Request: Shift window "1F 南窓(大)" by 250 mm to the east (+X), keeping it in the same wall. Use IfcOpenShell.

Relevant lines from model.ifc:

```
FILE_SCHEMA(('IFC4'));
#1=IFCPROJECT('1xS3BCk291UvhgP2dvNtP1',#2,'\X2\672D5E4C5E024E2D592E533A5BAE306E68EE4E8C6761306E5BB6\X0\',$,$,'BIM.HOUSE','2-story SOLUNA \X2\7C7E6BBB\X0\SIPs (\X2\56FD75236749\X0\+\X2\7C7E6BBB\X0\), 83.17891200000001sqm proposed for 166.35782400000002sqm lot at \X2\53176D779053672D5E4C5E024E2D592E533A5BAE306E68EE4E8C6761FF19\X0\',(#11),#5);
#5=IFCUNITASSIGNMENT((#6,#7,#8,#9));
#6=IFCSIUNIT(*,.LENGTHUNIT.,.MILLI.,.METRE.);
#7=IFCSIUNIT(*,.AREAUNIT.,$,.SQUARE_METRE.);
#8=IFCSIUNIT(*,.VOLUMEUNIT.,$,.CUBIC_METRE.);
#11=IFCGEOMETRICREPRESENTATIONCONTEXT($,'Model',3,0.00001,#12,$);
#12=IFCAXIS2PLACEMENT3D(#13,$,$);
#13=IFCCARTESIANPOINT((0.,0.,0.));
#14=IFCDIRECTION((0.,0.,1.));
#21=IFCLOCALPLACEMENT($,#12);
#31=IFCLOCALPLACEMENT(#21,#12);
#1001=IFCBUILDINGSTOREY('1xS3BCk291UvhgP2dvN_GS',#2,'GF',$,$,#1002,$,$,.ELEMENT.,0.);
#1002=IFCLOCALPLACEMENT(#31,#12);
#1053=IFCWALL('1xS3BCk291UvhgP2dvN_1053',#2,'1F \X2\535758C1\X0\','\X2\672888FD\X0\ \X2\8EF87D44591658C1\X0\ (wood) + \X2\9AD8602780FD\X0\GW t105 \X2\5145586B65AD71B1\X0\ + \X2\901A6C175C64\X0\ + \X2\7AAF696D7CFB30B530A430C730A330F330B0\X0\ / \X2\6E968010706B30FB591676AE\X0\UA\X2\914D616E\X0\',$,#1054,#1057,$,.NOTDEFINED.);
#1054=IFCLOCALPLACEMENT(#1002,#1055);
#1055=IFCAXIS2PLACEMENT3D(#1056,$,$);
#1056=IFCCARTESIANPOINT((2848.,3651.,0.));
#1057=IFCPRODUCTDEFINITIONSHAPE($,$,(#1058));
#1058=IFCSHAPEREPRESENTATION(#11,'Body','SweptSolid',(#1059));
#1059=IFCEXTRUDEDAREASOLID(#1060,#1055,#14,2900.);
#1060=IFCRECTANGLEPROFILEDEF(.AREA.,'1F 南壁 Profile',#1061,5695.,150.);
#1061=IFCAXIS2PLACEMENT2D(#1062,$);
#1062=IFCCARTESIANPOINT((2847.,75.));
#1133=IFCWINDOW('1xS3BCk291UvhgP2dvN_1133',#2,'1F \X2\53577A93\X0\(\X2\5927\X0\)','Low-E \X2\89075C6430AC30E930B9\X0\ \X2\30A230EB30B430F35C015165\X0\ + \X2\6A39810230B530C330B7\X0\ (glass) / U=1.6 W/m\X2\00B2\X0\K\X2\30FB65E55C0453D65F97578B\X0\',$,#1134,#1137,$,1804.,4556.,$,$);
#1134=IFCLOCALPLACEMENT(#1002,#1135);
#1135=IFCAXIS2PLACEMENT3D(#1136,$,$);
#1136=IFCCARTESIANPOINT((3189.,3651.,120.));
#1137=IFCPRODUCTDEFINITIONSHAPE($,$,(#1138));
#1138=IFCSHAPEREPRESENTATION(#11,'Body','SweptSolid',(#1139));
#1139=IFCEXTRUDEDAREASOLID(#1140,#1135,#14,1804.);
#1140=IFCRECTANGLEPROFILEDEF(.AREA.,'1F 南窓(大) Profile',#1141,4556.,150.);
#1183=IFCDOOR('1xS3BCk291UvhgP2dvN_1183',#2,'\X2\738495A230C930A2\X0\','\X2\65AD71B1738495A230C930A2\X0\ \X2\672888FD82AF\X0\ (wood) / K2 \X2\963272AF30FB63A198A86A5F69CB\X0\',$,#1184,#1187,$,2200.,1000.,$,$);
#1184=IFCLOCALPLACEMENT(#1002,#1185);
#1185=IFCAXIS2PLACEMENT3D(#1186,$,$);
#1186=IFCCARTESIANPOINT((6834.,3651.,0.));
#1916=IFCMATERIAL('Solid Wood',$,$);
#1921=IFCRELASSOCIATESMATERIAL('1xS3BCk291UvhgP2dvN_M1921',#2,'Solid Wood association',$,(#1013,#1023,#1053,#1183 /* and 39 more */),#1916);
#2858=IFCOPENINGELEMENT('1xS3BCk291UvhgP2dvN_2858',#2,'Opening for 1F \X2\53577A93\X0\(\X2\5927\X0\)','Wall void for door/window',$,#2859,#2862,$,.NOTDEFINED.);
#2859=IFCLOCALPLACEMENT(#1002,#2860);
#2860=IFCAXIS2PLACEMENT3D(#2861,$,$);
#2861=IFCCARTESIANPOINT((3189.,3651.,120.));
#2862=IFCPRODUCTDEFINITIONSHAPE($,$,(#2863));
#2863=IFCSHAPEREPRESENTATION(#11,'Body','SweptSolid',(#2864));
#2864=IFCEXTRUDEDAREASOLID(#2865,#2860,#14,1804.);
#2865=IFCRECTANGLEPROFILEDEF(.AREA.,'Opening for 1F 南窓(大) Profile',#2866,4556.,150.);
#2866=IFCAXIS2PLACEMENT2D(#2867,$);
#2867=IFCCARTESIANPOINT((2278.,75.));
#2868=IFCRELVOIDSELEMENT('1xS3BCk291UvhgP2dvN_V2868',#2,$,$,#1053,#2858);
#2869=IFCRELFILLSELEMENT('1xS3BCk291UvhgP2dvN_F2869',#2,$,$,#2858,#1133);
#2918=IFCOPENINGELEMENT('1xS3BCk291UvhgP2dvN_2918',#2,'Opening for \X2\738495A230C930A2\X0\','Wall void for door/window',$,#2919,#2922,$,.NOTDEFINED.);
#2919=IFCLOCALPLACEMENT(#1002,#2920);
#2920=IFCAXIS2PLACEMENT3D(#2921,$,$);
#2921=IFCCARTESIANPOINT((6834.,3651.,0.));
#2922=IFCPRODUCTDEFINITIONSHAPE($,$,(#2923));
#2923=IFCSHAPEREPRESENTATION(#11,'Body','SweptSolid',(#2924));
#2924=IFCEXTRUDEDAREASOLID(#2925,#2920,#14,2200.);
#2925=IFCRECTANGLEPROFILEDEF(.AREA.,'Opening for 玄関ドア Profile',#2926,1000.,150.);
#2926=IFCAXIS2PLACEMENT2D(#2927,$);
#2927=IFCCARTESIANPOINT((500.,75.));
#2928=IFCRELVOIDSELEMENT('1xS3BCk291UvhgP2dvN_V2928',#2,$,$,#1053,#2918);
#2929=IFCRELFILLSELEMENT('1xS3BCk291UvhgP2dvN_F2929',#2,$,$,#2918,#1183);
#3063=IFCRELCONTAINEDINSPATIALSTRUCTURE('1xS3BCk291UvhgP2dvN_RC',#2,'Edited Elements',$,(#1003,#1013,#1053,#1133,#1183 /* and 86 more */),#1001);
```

```python
import ifcopenshell
import ifcopenshell.api.geometry
import ifcopenshell.util.placement

model = ifcopenshell.open("model.ifc")

window = model.by_guid("1xS3BCk291UvhgP2dvN_1133")
opening = window.FillsVoids[0].RelatingOpeningElement
wall = opening.VoidsElements[0].RelatingBuildingElement

wall_matrix = ifcopenshell.util.placement.get_local_placement(wall.ObjectPlacement)
shift = wall_matrix[:3, 0] * 250.0
before = ifcopenshell.util.placement.get_local_placement(window.ObjectPlacement)[:3, 3].copy()

# The window is not placed relative to its opening, so move both.
for product in (opening, window):
    matrix = ifcopenshell.util.placement.get_local_placement(product.ObjectPlacement)
    matrix[:3, 3] += shift
    ifcopenshell.api.geometry.edit_object_placement(model, product=product, matrix=matrix, is_si=False)

after = ifcopenshell.util.placement.get_local_placement(window.ObjectPlacement)[:3, 3]
print("window moved by", (after - before).round(3) + 0.0)

model.write("model_updated.ifc")
```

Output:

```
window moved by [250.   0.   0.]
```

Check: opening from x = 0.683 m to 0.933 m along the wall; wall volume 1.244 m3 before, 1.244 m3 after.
